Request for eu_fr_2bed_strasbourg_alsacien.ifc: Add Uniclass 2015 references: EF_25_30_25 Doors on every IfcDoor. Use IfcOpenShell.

First a look at what the model holds.

```python
import ifcopenshell

model = ifcopenshell.open("eu_fr_2bed_strasbourg_alsacien.ifc")
print(model.schema)
print("classifications:", [c.Name for c in model.by_type("IfcClassification")])
for ifc_class in ("IfcDoor", "IfcRoof", "IfcStair", "IfcWall", "IfcWindow"):
    print(ifc_class, len(model.by_type(ifc_class)))
```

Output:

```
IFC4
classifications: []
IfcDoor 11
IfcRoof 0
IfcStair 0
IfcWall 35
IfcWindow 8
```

```python
import ifcopenshell
import ifcopenshell.api.classification

model = ifcopenshell.open("eu_fr_2bed_strasbourg_alsacien.ifc")

system = ifcopenshell.api.classification.add_classification(model, classification="Uniclass 2015")

codes = {
    "IfcDoor": ("EF_25_30_25", "Doors"),
}
for ifc_class, (code, name) in codes.items():
    products = model.by_type(ifc_class)
    ifcopenshell.api.classification.add_reference(
        model, products=products, classification=system, identification=code, name=name
    )
    print(code, len(products))

model.write("eu_fr_2bed_strasbourg_alsacien_rev.ifc")
```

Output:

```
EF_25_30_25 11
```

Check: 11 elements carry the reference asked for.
